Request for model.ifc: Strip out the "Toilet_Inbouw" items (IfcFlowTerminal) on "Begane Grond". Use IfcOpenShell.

First a look at what the model holds.

```python
import ifcopenshell
import ifcopenshell.util.element

model = ifcopenshell.open("model.ifc")
print(model.schema)
storey = next(s for s in model.by_type("IfcBuildingStorey") if s.Name == "Begane Grond")
terminals = [e for e in ifcopenshell.util.element.get_decomposition(storey) if e.is_a("IfcFlowTerminal")]
seen = {}
for e in terminals:
    element_type = ifcopenshell.util.element.get_type(e)
    name = element_type.Name if element_type not in (None, e) else None
    seen[name] = seen.get(name, 0) + 1
for name, count in sorted(seen.items(), key=str):
    print(count, "x", name)
```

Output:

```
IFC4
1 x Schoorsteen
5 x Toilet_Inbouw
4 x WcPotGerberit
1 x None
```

```python
import ifcopenshell
import ifcopenshell.api.root
import ifcopenshell.util.element

model = ifcopenshell.open("model.ifc")

storey = next(s for s in model.by_type("IfcBuildingStorey") if s.Name == "Begane Grond")
terminals = [e for e in ifcopenshell.util.element.get_decomposition(storey) if e.is_a("IfcFlowTerminal")]
targets = [e for e in terminals if (t := ifcopenshell.util.element.get_type(e)) not in (None, e) and t.Name == "Toilet_Inbouw"]

for e in targets:
    ifcopenshell.api.root.remove_product(model, product=e)
print(len(targets), "removed")

model.write("model_edited.ifc")
```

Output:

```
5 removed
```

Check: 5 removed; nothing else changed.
